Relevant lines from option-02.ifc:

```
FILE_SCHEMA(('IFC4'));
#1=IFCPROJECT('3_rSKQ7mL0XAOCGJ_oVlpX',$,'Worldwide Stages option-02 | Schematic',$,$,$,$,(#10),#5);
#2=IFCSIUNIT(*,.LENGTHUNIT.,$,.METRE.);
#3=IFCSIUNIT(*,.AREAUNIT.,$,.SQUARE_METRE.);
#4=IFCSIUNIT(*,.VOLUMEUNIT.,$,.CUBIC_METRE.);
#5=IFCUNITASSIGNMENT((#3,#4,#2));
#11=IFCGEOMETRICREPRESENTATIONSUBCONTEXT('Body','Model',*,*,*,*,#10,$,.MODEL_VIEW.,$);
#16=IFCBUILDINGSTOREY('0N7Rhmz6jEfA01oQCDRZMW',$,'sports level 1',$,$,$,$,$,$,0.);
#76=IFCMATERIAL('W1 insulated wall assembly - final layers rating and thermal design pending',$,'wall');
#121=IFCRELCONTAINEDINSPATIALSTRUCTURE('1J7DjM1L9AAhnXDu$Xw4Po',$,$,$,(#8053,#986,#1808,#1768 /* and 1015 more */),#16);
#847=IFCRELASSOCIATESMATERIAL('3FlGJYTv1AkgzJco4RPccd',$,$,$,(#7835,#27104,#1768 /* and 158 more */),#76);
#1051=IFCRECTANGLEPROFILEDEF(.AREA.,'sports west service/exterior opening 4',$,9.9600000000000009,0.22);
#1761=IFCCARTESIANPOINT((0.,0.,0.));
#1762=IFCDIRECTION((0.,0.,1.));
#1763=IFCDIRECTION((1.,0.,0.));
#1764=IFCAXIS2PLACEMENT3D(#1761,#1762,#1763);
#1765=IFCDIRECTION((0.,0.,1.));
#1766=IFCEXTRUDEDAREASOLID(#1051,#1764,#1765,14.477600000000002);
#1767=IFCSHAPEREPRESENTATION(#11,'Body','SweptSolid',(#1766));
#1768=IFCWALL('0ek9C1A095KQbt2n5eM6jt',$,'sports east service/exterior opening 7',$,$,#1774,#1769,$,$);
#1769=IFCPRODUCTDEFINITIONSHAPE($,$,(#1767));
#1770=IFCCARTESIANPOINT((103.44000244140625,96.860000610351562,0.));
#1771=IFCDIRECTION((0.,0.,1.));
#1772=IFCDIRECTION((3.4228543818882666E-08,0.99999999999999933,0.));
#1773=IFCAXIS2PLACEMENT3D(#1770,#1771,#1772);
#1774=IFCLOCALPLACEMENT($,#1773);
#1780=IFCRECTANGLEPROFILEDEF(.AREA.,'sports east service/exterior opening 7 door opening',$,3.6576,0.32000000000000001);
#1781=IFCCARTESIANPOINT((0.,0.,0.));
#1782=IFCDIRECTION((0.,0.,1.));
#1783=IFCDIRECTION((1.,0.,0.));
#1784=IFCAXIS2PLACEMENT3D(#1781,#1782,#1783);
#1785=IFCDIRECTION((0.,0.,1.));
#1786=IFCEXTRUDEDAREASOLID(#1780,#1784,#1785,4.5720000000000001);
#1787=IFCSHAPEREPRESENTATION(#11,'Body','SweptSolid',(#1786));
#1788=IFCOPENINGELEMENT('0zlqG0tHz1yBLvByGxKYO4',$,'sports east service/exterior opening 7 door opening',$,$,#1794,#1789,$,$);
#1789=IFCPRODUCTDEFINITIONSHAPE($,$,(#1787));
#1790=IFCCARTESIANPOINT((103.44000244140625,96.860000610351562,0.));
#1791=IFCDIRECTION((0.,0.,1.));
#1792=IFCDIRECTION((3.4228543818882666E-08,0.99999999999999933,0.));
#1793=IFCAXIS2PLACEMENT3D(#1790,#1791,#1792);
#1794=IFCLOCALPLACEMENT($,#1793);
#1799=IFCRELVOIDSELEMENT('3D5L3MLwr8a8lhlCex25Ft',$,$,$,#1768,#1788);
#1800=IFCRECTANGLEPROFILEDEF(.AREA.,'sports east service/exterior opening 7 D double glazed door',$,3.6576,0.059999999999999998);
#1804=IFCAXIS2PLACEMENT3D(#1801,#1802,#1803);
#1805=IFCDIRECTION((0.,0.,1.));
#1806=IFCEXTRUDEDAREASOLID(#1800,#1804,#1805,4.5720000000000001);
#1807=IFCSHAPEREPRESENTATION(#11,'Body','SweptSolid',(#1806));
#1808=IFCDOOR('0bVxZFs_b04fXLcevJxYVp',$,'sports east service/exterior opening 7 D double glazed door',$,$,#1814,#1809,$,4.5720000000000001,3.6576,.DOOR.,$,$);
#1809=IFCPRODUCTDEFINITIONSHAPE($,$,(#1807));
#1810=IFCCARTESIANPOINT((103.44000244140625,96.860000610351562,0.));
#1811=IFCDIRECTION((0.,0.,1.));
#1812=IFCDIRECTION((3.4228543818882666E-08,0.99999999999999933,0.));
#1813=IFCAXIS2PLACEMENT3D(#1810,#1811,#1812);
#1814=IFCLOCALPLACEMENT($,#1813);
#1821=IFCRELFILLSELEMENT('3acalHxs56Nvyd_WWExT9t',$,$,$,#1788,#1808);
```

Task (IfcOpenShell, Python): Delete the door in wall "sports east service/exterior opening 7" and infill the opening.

```python
import ifcopenshell
import ifcopenshell.api.feature
import ifcopenshell.api.root
import ifcopenshell.geom
import ifcopenshell.util.shape

model = ifcopenshell.open("option-02.ifc")
settings = ifcopenshell.geom.settings()


def volume(element):
    """Net volume in cubic metres, openings subtracted."""
    shape = ifcopenshell.geom.create_shape(settings, element)
    return ifcopenshell.util.shape.get_volume(shape.geometry)


door = model.by_guid("0bVxZFs_b04fXLcevJxYVp")
opening = door.FillsVoids[0].RelatingOpeningElement
wall = opening.VoidsElements[0].RelatingBuildingElement
before = volume(wall)

ifcopenshell.api.root.remove_product(model, product=door)
ifcopenshell.api.feature.remove_feature(model, feature=opening)

after = volume(wall)

print(f"wall volume {before:.3f} -> {after:.3f} m3")

model.write("option-02-out.ifc")
```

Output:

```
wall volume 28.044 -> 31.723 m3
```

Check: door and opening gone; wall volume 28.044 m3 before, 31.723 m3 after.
